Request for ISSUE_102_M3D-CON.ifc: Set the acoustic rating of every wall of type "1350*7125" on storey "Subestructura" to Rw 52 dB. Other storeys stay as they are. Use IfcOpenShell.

First a look at what the model holds.

```python
import ifcopenshell
import ifcopenshell.util.element

model = ifcopenshell.open("ISSUE_102_M3D-CON.ifc")
print(model.schema)
storey = next(s for s in model.by_type("IfcBuildingStorey") if s.Name == "Subestructura")
walls = [e for e in ifcopenshell.util.element.get_decomposition(storey) if e.is_a("IfcWall")]
seen = {}
for e in walls:
    element_type = ifcopenshell.util.element.get_type(e)
    key = (element_type.Name if element_type != e and element_type else None, ifcopenshell.util.element.get_pset(e, "Pset_WallCommon", "AcousticRating"))
    seen[key] = seen.get(key, 0) + 1
for (name, value), count in sorted(seen.items(), key=str):
    print(count, "x", name, "|", value)
```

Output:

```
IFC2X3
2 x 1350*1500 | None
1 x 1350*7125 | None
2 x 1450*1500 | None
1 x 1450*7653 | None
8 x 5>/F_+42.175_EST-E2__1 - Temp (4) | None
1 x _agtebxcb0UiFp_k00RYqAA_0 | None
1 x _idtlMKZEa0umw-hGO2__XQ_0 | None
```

```python
import ifcopenshell
import ifcopenshell.api.pset
import ifcopenshell.util.element

model = ifcopenshell.open("ISSUE_102_M3D-CON.ifc")

storey = next(s for s in model.by_type("IfcBuildingStorey") if s.Name == "Subestructura")
walls = [e for e in ifcopenshell.util.element.get_decomposition(storey) if e.is_a("IfcWall")]

count = 0
for e in walls:
    element_type = ifcopenshell.util.element.get_type(e)
    if element_type in (None, e) or element_type.Name != "1350*7125":
        continue
    # add_pset returns the element's existing set when there is one.
    pset = ifcopenshell.api.pset.add_pset(model, product=e, name="Pset_WallCommon")
    ifcopenshell.api.pset.edit_pset(model, pset=pset, properties={"AcousticRating": "Rw 52 dB"})
    count += 1

print(count, "walls updated")

model.write("ISSUE_102_M3D-CON_updated.ifc")
```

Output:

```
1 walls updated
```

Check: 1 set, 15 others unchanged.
